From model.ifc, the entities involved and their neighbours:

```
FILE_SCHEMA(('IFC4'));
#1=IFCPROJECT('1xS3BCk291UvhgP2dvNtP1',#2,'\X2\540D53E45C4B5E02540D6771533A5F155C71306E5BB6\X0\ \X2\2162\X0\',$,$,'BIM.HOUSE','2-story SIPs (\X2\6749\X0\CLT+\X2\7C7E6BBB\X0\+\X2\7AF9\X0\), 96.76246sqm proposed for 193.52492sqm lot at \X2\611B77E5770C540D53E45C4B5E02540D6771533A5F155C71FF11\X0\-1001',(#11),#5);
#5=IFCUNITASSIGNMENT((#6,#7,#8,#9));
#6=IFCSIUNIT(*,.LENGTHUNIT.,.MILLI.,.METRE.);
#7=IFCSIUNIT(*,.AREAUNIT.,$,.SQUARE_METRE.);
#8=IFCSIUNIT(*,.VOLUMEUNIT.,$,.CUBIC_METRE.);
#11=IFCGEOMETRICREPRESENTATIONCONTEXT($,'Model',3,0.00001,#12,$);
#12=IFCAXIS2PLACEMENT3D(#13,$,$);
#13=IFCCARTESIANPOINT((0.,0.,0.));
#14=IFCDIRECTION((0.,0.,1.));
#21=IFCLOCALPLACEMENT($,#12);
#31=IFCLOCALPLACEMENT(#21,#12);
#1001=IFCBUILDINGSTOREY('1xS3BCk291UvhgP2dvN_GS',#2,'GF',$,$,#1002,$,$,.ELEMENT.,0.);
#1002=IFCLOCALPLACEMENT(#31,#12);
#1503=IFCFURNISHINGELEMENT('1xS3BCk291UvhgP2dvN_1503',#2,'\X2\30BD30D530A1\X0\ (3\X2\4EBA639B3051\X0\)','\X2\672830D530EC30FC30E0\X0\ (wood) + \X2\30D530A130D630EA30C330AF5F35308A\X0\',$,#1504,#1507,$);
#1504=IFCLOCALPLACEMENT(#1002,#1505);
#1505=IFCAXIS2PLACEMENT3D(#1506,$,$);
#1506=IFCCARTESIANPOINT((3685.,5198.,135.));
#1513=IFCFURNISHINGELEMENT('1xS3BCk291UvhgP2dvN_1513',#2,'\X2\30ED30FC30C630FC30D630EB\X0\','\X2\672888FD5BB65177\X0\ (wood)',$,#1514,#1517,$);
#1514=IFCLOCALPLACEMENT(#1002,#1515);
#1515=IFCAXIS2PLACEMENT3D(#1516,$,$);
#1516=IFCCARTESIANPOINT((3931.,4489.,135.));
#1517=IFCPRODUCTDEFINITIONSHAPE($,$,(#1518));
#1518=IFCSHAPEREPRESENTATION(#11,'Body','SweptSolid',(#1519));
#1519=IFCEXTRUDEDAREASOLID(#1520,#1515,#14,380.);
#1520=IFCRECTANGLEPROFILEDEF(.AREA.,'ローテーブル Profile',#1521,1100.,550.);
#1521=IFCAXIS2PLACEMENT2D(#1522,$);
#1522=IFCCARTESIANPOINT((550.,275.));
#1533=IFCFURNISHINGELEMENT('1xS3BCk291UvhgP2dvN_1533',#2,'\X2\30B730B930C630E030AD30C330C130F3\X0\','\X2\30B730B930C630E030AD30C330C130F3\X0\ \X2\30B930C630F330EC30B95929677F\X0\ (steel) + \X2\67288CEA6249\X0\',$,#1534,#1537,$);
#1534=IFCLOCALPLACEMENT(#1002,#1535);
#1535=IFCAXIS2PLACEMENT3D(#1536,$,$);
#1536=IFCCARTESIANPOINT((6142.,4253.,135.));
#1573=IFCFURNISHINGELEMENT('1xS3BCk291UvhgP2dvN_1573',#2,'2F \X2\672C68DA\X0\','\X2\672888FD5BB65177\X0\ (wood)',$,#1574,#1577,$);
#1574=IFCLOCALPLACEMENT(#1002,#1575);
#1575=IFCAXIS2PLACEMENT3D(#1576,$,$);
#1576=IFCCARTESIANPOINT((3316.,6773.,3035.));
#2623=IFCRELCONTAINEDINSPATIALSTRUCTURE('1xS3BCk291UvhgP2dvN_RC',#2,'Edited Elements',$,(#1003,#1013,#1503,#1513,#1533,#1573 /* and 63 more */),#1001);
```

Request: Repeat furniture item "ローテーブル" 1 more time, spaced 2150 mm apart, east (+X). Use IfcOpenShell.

```python
import numpy as np
import ifcopenshell
import ifcopenshell.api.geometry
import ifcopenshell.api.root
import ifcopenshell.util.element
import ifcopenshell.util.placement

model = ifcopenshell.open("model.ifc")


def reuse_history(source, copy):
    """copy_class also copies each property set's owner history, people and application; keep the originals."""
    for rel in copy.IsDefinedBy:
        if rel.is_a("IfcRelDefinesByProperties") and (history := rel.RelatingPropertyDefinition.OwnerHistory):
            rel.RelatingPropertyDefinition.OwnerHistory = source.OwnerHistory
            ifcopenshell.util.element.remove_deep2(model, history)


source = model.by_id(1513)
base = ifcopenshell.util.placement.get_local_placement(source.ObjectPlacement)
step = np.array([1.0, 0.0, 0.0]) * 2150.0

for i in range(1, 2):
    copy = ifcopenshell.api.root.copy_class(model, product=source)
    copy.Representation = ifcopenshell.util.element.copy_deep(
        model, source.Representation, exclude=["IfcGeometricRepresentationContext", "IfcRepresentationMap"]
    )
    reuse_history(source, copy)
    matrix = base.copy()
    matrix[:3, 3] += i * step
    print("added at", matrix[:3, 3].round(3) + 0.0)
    ifcopenshell.api.geometry.edit_object_placement(model, product=copy, matrix=matrix, is_si=False)

model.write("model-out.ifc")
```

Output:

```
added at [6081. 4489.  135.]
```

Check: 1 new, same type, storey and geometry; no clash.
